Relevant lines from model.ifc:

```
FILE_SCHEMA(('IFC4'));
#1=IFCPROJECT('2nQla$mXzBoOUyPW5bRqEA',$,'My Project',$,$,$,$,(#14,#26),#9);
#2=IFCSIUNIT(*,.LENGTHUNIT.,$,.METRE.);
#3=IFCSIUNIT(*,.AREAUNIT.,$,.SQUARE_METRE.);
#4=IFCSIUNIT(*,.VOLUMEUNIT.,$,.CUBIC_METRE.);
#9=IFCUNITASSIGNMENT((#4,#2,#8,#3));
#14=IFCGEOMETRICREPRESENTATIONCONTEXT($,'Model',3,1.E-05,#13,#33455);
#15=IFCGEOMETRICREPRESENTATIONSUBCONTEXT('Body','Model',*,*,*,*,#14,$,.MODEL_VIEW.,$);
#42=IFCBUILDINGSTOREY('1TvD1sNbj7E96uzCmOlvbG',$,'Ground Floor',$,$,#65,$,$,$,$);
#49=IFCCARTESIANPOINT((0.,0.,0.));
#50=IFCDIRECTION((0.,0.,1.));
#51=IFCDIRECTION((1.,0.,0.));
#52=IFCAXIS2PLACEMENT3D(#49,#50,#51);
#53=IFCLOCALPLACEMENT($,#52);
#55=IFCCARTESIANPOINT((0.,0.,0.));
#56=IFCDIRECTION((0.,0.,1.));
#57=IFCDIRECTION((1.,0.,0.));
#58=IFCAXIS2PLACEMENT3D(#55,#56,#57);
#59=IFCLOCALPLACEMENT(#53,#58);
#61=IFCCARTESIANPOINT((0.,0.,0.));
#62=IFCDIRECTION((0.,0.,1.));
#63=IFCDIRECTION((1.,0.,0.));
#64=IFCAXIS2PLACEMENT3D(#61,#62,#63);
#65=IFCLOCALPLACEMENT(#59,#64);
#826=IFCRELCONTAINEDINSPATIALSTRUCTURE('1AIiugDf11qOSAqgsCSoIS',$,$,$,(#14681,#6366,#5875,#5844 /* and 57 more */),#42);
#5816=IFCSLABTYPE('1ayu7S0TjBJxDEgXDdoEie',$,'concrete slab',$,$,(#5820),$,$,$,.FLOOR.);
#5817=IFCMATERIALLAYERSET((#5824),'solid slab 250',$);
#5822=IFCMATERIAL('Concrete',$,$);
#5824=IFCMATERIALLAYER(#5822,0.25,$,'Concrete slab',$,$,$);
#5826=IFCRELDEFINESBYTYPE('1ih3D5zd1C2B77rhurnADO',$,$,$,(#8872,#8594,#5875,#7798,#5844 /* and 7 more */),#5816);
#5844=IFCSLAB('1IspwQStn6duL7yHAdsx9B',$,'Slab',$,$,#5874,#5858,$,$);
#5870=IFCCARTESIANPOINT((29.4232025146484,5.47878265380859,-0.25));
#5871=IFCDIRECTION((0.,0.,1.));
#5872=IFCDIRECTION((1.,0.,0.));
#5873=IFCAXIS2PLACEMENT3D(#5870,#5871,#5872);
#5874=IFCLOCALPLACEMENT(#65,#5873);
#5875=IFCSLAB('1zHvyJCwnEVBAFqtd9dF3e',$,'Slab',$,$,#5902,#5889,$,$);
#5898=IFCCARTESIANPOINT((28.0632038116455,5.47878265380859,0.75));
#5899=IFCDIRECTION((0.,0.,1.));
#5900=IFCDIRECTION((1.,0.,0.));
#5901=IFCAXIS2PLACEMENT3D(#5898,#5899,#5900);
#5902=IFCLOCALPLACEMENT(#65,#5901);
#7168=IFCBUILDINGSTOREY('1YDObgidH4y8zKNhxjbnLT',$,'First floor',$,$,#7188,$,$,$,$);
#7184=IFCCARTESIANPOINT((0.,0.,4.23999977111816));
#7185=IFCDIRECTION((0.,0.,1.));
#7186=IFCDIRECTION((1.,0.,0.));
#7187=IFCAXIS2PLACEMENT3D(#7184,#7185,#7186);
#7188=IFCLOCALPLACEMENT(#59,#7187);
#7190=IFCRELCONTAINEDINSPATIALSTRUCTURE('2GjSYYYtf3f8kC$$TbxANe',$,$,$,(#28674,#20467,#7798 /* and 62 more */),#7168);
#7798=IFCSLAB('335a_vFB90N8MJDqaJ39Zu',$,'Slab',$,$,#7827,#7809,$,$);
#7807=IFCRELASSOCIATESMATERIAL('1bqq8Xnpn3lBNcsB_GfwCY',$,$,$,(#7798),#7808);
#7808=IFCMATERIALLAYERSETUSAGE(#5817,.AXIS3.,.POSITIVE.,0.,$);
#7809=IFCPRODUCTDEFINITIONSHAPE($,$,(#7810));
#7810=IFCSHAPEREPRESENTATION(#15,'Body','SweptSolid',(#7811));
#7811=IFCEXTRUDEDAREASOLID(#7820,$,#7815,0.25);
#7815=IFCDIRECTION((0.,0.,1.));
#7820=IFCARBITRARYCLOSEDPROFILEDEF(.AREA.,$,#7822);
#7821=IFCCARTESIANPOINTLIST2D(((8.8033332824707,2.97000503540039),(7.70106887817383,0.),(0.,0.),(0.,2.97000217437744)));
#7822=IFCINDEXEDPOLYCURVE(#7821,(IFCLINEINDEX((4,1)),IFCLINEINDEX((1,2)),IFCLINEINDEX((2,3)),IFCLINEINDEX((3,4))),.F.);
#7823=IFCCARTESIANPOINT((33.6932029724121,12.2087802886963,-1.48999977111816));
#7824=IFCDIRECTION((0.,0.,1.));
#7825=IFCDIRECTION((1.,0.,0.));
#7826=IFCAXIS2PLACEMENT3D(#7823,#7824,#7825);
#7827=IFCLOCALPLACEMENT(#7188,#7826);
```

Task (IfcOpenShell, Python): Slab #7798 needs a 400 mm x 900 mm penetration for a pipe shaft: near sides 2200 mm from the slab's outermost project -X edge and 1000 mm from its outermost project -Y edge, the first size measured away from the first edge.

```python
import numpy as np
import ifcopenshell
import ifcopenshell.api.feature
import ifcopenshell.api.geometry
import ifcopenshell.api.root
import ifcopenshell.geom
import ifcopenshell.util.placement
import ifcopenshell.util.representation
import ifcopenshell.util.shape
import ifcopenshell.util.unit

model = ifcopenshell.open("model.ifc")
unit_scale = ifcopenshell.util.unit.calculate_unit_scale(model)
settings = ifcopenshell.geom.settings()


def volume(element):
    """Net volume in cubic metres, openings subtracted."""
    shape = ifcopenshell.geom.create_shape(settings, element)
    return ifcopenshell.util.shape.get_volume(shape.geometry)


slab = model.by_id(7798)
before = volume(slab)

# Extent in the slab's own axes, in metres. The edges named are its -X and -Y sides.
slab_shape = ifcopenshell.geom.create_shape(settings, slab)
vertices = ifcopenshell.util.shape.get_vertices(slab_shape.geometry)
x_min, y_min, bottom = vertices.min(axis=0)
top = vertices[:, 2].max()

opening = ifcopenshell.api.root.create_entity(model, ifc_class="IfcOpeningElement", name="Pipe shaft opening", predefined_type="OPENING")
context = ifcopenshell.util.representation.get_context(model, "Model", "Body", "MODEL_VIEW")
width, depth = 0.4, 0.9
outline = [(0.0, 0.0), (width, 0.0), (width, depth), (0.0, depth), (0.0, 0.0)]
# Overshoot both faces by 50 mm so the cut is clean.
shape = ifcopenshell.api.geometry.add_slab_representation(
    model, context=context, depth=top - bottom + 0.1, polyline=outline
)
ifcopenshell.api.geometry.assign_representation(model, product=opening, representation=shape)

matrix = ifcopenshell.util.placement.get_local_placement(slab.ObjectPlacement)
matrix[:, 3] = matrix @ np.append(np.array([x_min + 2.2, y_min + 1, bottom - 0.05]) / unit_scale, 1.0)
ifcopenshell.api.geometry.edit_object_placement(model, product=opening, matrix=matrix, is_si=False)
ifcopenshell.api.feature.add_feature(model, feature=opening, element=slab)

after = volume(slab)

print(f"slab volume {before:.3f} -> {after:.3f} m3")

model.write("model_v2.ifc")
```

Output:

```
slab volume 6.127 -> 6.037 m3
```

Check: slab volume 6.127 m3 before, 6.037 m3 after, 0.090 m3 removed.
